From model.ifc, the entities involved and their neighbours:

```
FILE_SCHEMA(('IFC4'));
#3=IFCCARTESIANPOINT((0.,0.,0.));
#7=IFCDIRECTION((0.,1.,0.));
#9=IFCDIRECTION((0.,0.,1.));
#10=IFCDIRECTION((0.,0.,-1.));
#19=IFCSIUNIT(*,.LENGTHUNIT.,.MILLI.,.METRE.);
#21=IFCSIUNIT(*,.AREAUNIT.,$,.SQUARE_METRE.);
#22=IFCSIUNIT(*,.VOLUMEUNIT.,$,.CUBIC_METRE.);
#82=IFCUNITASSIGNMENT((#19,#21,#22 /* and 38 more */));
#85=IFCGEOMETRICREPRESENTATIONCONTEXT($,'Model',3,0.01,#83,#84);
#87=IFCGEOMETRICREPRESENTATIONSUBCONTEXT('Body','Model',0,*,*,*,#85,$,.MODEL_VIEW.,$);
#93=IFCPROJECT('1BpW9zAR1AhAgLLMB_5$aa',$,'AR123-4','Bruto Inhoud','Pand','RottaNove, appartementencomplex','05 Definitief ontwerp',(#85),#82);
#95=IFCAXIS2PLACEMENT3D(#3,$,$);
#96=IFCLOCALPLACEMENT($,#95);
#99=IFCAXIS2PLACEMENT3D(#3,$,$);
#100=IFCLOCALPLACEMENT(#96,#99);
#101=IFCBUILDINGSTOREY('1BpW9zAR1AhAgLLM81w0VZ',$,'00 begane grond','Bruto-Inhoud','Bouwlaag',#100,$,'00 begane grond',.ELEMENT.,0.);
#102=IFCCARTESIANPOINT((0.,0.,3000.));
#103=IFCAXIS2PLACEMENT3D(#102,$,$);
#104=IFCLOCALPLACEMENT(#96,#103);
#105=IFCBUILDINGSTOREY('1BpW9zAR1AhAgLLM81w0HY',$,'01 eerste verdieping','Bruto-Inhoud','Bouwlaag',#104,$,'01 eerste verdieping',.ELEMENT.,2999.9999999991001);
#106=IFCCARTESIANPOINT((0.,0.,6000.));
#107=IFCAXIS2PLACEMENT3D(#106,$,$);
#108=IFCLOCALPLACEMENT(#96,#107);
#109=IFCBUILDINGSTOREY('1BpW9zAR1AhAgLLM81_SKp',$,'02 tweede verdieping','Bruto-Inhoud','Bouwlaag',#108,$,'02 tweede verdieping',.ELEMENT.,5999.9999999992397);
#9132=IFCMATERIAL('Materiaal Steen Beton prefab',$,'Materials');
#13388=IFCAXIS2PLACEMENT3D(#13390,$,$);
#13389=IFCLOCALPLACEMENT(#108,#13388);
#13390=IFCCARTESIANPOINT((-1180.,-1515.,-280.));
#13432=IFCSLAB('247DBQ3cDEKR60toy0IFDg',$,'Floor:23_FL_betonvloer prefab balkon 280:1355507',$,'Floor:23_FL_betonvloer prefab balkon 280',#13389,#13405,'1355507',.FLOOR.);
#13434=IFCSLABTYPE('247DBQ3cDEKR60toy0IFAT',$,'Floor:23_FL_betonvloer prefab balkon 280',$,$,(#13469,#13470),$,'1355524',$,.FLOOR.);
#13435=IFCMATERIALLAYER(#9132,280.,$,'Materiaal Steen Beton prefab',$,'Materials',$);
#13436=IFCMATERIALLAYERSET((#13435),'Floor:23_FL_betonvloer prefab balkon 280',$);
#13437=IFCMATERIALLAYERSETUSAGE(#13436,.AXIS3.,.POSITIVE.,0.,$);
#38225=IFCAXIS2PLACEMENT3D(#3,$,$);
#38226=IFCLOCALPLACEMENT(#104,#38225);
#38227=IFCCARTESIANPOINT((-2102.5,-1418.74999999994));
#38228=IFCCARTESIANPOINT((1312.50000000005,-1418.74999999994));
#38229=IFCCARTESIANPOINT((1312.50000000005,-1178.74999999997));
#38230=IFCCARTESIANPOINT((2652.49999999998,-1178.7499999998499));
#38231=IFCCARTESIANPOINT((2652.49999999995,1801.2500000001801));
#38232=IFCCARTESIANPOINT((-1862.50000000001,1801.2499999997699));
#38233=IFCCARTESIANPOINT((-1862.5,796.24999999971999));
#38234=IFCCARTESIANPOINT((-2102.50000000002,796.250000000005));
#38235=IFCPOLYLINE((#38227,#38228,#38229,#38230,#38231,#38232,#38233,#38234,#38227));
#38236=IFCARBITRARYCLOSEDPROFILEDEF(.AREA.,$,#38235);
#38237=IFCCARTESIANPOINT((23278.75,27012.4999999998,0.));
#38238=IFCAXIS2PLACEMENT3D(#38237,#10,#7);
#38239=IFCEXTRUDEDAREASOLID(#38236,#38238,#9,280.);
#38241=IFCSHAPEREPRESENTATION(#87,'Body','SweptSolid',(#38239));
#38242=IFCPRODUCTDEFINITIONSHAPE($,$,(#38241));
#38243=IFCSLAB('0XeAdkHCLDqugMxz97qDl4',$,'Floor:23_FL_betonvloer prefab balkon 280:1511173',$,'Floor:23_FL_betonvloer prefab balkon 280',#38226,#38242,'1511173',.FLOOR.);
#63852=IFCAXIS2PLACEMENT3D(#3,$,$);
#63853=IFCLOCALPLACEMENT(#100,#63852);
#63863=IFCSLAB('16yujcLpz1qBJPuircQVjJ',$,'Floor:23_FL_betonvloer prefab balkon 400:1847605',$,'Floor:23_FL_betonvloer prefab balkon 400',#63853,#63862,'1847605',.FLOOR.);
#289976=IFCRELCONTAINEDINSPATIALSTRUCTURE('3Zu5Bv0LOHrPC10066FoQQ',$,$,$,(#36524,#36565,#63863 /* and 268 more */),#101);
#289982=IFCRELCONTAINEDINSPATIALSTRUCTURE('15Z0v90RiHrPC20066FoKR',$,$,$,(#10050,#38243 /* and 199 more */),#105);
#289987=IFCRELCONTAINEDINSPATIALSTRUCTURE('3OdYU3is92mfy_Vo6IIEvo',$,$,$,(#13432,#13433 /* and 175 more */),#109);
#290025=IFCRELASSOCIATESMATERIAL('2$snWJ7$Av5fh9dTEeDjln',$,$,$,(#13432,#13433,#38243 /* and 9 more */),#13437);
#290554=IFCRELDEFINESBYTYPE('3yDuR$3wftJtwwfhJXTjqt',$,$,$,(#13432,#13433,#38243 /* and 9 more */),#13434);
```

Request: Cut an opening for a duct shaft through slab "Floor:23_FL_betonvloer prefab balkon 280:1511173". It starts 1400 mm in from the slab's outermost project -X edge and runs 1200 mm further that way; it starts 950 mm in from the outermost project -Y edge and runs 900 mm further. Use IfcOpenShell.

```python
import numpy as np
import ifcopenshell
import ifcopenshell.api.feature
import ifcopenshell.api.geometry
import ifcopenshell.api.root
import ifcopenshell.geom
import ifcopenshell.util.placement
import ifcopenshell.util.representation
import ifcopenshell.util.shape
import ifcopenshell.util.unit

model = ifcopenshell.open("model.ifc")
unit_scale = ifcopenshell.util.unit.calculate_unit_scale(model)
settings = ifcopenshell.geom.settings()


def volume(element):
    """Net volume in cubic metres, openings subtracted."""
    shape = ifcopenshell.geom.create_shape(settings, element)
    return ifcopenshell.util.shape.get_volume(shape.geometry)


slab = model.by_guid("0XeAdkHCLDqugMxz97qDl4")
before = volume(slab)

# Extent in the slab's own axes, in metres. The edges named are its -X and -Y sides.
slab_shape = ifcopenshell.geom.create_shape(settings, slab)
vertices = ifcopenshell.util.shape.get_vertices(slab_shape.geometry)
x_min, y_min, bottom = vertices.min(axis=0)
top = vertices[:, 2].max()

opening = ifcopenshell.api.root.create_entity(model, ifc_class="IfcOpeningElement", name="Duct shaft opening", predefined_type="OPENING")
context = ifcopenshell.util.representation.get_context(model, "Model", "Body", "MODEL_VIEW")
width, depth = 1.2, 0.9
outline = [(0.0, 0.0), (width, 0.0), (width, depth), (0.0, depth), (0.0, 0.0)]
# Overshoot both faces by 50 mm so the cut is clean.
shape = ifcopenshell.api.geometry.add_slab_representation(
    model, context=context, depth=top - bottom + 0.1, polyline=outline
)
ifcopenshell.api.geometry.assign_representation(model, product=opening, representation=shape)

matrix = ifcopenshell.util.placement.get_local_placement(slab.ObjectPlacement)
matrix[:, 3] = matrix @ np.append(np.array([x_min + 1.4, y_min + 0.95, bottom - 0.05]) / unit_scale, 1.0)
ifcopenshell.api.geometry.edit_object_placement(model, product=opening, matrix=matrix, is_si=False)
ifcopenshell.api.feature.add_feature(model, feature=opening, element=slab)

after = volume(slab)

print(f"slab volume {before:.3f} -> {after:.3f} m3")

model.write("model_v2.ifc")
```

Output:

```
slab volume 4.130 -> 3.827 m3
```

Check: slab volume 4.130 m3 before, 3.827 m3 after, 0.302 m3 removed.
